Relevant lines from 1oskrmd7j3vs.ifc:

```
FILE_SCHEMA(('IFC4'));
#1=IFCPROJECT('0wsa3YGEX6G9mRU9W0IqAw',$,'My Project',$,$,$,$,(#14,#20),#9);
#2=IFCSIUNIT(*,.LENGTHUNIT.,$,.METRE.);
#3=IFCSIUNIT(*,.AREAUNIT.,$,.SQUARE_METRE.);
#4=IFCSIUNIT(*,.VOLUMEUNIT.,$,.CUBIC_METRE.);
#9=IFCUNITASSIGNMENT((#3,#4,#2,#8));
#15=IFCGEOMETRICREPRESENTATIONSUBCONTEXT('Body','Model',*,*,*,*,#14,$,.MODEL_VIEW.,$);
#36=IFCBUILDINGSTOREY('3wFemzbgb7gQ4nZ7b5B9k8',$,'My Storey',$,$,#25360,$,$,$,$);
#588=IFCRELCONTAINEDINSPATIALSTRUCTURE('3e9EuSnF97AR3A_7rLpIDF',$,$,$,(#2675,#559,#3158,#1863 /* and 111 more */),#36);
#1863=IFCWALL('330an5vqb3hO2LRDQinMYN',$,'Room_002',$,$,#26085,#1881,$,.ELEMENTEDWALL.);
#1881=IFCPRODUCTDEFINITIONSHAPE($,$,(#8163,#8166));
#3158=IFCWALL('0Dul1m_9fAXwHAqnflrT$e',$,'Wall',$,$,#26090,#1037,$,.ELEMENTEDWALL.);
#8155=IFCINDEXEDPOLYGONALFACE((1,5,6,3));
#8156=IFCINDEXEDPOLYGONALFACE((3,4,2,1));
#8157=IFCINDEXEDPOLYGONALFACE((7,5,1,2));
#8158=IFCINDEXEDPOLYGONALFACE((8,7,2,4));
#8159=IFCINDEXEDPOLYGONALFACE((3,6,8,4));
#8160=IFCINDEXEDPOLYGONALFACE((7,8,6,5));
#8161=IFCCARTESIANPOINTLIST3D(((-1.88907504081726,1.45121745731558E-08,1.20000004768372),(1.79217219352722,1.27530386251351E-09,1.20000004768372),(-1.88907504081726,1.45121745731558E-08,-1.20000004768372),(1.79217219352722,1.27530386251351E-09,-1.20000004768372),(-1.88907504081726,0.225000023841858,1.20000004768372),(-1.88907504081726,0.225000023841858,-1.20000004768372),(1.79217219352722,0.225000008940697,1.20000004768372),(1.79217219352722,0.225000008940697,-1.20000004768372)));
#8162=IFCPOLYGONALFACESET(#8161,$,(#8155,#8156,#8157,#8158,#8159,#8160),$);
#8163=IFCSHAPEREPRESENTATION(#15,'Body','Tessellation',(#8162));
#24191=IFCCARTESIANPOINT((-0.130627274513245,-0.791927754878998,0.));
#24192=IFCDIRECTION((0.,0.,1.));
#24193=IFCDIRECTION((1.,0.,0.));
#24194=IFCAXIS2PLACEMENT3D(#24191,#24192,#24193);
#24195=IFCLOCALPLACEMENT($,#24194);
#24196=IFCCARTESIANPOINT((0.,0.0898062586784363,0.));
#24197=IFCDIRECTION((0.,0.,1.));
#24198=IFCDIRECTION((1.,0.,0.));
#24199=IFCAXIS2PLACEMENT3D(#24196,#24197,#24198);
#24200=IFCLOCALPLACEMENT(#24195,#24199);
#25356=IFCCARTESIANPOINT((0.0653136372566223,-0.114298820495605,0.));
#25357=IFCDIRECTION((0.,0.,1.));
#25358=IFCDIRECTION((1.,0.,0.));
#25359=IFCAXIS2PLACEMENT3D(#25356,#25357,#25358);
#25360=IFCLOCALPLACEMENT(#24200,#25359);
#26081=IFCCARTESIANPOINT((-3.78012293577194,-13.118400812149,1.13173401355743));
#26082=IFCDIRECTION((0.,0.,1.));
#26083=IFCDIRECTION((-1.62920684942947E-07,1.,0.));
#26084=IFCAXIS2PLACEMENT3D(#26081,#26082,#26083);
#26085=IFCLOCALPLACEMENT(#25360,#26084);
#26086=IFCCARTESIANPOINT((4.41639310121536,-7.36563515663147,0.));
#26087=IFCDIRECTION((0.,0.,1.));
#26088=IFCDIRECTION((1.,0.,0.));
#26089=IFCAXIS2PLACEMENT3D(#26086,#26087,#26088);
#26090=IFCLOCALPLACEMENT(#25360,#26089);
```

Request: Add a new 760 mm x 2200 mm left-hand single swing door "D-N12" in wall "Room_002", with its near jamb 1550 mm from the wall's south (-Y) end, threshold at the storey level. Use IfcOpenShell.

```python
import numpy as np
import ifcopenshell
import ifcopenshell.api.feature
import ifcopenshell.api.geometry
import ifcopenshell.api.root
import ifcopenshell.api.spatial
import ifcopenshell.geom
import ifcopenshell.util.element
import ifcopenshell.util.placement
import ifcopenshell.util.representation
import ifcopenshell.util.shape
import ifcopenshell.util.unit

model = ifcopenshell.open("1oskrmd7j3vs.ifc")
unit_scale = ifcopenshell.util.unit.calculate_unit_scale(model)
settings = ifcopenshell.geom.settings()


def volume(element):
    """Net volume in cubic metres, openings subtracted."""
    shape = ifcopenshell.geom.create_shape(settings, element)
    return ifcopenshell.util.shape.get_volume(shape.geometry)


wall = model.by_guid("330an5vqb3hO2LRDQinMYN")
storey = ifcopenshell.util.element.get_container(wall, ifc_class="IfcBuildingStorey")
context = ifcopenshell.util.representation.get_context(model, "Model", "Body", "MODEL_VIEW")
before = volume(wall)

width, height, from_end, sill = 0.76, 2.2, 1.55, 0.0  # metres

# The wall runs along its own X axis, and the end named is its -X end.
wall_shape = ifcopenshell.geom.create_shape(settings, wall)
x, y, z = ifcopenshell.util.shape.get_vertices(wall_shape.geometry).T
start = x.min() + from_end
face, thickness = float(y.min()), float(y.max() - y.min())
wall_matrix = ifcopenshell.util.placement.get_local_placement(wall.ObjectPlacement)
level = ifcopenshell.util.placement.get_local_placement(storey.ObjectPlacement)[2, 3]


def in_wall(x, y):
    """Placement at x, y metres in the wall's axes, at sill height."""
    matrix = wall_matrix.copy()
    matrix[:, 3] = wall_matrix @ np.array([x / unit_scale, y / unit_scale, 0.0, 1.0])
    matrix[2, 3] = level + sill / unit_scale
    return matrix


# Opening: a box that overshoots both wall faces by 50 mm.
opening = ifcopenshell.api.root.create_entity(model, ifc_class="IfcOpeningElement", predefined_type="OPENING")
box = ifcopenshell.api.geometry.add_wall_representation(
    model, context=context, length=width, height=height, thickness=thickness + 0.1
)
ifcopenshell.api.geometry.assign_representation(model, product=opening, representation=box)
ifcopenshell.api.geometry.edit_object_placement(model, product=opening, matrix=in_wall(start, face - 0.05), is_si=False)
ifcopenshell.api.feature.add_feature(model, feature=opening, element=wall)

door = ifcopenshell.api.root.create_entity(model, ifc_class="IfcDoor", name="D-N12", predefined_type="DOOR")
door.OverallWidth, door.OverallHeight = width / unit_scale, height / unit_scale
door.OperationType = "SINGLE_SWING_LEFT"
body = ifcopenshell.api.geometry.add_door_representation(
    model,
    context=context,
    overall_width=door.OverallWidth,
    overall_height=door.OverallHeight,
    operation_type="SINGLE_SWING_LEFT",
    lining_properties={"LiningDepth": thickness / unit_scale, "ThresholdDepth": thickness / unit_scale},
)
ifcopenshell.api.geometry.assign_representation(model, product=door, representation=body)
ifcopenshell.api.spatial.assign_container(model, products=[door], relating_structure=storey)
ifcopenshell.api.feature.add_filling(model, opening=opening, element=door)

# The lining spans the wall, so the door starts at the wall face.
ifcopenshell.api.geometry.edit_object_placement(model, product=door, matrix=in_wall(start, face), is_si=False)

after = volume(wall)

print(f"wall volume {before:.3f} -> {after:.3f} m3")

model.write("1oskrmd7j3vs_v2.ifc")
```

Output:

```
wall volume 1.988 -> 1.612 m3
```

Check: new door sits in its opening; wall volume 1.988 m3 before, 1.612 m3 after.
